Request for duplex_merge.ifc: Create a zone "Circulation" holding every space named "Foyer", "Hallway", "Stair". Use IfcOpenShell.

First a look at what the model holds.

```python
import ifcopenshell

model = ifcopenshell.open("duplex_merge.ifc")
print(model.schema)
seen = {}
for space in model.by_type("IfcSpace"):
    seen[space.LongName] = seen.get(space.LongName, 0) + 1
for name, count in sorted(seen.items(), key=str):
    print(count, "x", name)
print("zones:", [z.Name for z in model.by_type("IfcZone")][:20])
```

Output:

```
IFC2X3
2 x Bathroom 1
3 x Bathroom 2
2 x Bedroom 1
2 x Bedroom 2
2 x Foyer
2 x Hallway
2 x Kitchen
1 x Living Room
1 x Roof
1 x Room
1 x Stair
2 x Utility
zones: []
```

```python
import ifcopenshell
import ifcopenshell.api.group
import ifcopenshell.api.root

model = ifcopenshell.open("duplex_merge.ifc")

names = {"Foyer", "Hallway", "Stair"}
spaces = [s for s in model.by_type("IfcSpace") if s.LongName in names]

zone = ifcopenshell.api.root.create_entity(model, ifc_class="IfcZone", name="Circulation")
ifcopenshell.api.group.assign_group(model, products=spaces, group=zone)
print(len(spaces), "spaces in", zone.Name)

model.write("duplex_merge_edited.ifc")
```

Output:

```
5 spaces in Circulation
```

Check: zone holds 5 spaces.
